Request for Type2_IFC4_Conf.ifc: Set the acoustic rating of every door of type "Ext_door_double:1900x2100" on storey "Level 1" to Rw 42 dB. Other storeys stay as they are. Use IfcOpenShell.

First a look at what the model holds.

```python
import ifcopenshell
import ifcopenshell.util.element

model = ifcopenshell.open("Type2_IFC4_Conf.ifc")
print(model.schema)
storey = next(s for s in model.by_type("IfcBuildingStorey") if s.Name == "Level 1")
doors = [e for e in ifcopenshell.util.element.get_decomposition(storey) if e.is_a("IfcDoor")]
seen = {}
for e in doors:
    element_type = ifcopenshell.util.element.get_type(e)
    key = (element_type.Name if element_type != e and element_type else None, ifcopenshell.util.element.get_pset(e, "Pset_DoorCommon", "AcousticRating"))
    seen[key] = seen.get(key, 0) + 1
for (name, value), count in sorted(seen.items(), key=str):
    print(count, "x", name, "|", value)
```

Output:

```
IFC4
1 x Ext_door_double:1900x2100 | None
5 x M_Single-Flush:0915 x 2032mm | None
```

```python
import ifcopenshell
import ifcopenshell.api.pset
import ifcopenshell.util.element

model = ifcopenshell.open("Type2_IFC4_Conf.ifc")

storey = next(s for s in model.by_type("IfcBuildingStorey") if s.Name == "Level 1")
doors = [e for e in ifcopenshell.util.element.get_decomposition(storey) if e.is_a("IfcDoor")]

count = 0
for e in doors:
    element_type = ifcopenshell.util.element.get_type(e)
    if element_type in (None, e) or element_type.Name != "Ext_door_double:1900x2100":
        continue
    # add_pset returns the element's existing set when there is one.
    pset = ifcopenshell.api.pset.add_pset(model, product=e, name="Pset_DoorCommon")
    ifcopenshell.api.pset.edit_pset(model, pset=pset, properties={"AcousticRating": "Rw 42 dB"})
    count += 1

print(count, "doors updated")

model.write("Type2_IFC4_Conf-out.ifc")
```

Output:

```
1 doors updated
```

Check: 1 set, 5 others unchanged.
